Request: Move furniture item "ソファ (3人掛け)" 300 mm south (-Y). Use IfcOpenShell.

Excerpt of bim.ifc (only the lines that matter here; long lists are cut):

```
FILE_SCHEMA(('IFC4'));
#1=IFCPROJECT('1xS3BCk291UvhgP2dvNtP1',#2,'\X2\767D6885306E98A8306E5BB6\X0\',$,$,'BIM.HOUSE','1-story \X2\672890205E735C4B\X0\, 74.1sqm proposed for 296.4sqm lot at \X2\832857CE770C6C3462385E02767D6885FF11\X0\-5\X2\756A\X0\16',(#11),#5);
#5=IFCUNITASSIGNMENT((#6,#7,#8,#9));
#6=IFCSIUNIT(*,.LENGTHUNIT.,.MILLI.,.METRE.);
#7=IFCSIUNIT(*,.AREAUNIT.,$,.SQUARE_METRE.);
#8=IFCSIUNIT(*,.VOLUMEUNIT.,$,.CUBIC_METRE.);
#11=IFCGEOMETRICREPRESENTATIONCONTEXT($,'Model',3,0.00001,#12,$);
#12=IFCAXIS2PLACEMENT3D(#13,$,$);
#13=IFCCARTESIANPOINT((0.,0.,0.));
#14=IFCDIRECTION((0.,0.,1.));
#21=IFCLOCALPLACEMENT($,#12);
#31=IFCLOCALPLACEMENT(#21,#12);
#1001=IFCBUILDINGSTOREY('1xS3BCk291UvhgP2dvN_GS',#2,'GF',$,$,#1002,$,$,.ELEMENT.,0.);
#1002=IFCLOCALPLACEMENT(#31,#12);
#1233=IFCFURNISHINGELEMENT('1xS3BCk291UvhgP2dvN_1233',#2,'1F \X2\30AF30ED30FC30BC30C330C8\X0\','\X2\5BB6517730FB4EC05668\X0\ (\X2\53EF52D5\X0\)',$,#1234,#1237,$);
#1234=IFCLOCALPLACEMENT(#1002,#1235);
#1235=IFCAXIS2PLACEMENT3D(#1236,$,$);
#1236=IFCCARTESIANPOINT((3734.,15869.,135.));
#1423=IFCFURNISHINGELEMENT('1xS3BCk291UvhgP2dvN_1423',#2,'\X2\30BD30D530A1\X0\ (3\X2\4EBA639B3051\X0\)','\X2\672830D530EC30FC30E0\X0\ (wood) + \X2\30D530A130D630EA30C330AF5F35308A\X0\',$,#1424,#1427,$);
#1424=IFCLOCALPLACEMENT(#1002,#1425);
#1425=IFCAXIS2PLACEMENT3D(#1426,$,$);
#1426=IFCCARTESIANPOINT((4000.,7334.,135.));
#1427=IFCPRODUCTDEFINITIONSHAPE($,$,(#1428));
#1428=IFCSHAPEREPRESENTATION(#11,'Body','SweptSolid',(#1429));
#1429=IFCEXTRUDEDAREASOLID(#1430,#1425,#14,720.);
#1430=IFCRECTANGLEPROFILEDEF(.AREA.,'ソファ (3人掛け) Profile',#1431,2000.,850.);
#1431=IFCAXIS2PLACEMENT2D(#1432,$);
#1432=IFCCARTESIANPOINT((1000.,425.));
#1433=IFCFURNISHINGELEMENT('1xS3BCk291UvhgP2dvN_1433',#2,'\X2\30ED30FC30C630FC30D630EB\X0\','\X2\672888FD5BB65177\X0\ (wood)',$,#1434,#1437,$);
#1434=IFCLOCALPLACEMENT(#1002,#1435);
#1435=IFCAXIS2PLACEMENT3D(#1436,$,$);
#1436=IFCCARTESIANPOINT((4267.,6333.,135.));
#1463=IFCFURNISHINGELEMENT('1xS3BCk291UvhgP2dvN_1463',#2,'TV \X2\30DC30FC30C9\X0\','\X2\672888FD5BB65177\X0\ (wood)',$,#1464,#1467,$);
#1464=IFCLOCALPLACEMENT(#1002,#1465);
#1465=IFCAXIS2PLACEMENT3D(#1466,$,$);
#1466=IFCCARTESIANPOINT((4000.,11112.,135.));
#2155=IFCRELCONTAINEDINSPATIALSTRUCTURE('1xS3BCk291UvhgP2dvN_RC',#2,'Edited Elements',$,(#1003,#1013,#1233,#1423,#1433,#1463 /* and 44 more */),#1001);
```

```python
import ifcopenshell
import ifcopenshell.api.geometry
import ifcopenshell.util.placement
import ifcopenshell.util.unit

model = ifcopenshell.open("bim.ifc")
unit_scale = ifcopenshell.util.unit.calculate_unit_scale(model)

item = model.by_guid("1xS3BCk291UvhgP2dvN_1423")
matrix = ifcopenshell.util.placement.get_local_placement(item.ObjectPlacement)
matrix[1, 3] -= 0.3 / unit_scale
ifcopenshell.api.geometry.edit_object_placement(model, product=item, matrix=matrix, is_si=False)

print(ifcopenshell.util.placement.get_local_placement(item.ObjectPlacement).round(3) + 0.0)

model.write("bim_rev.ifc")
```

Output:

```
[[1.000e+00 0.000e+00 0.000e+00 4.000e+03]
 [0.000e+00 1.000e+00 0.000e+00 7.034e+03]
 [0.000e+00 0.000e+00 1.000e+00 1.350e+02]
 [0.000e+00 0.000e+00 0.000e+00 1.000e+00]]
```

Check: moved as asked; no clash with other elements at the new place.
